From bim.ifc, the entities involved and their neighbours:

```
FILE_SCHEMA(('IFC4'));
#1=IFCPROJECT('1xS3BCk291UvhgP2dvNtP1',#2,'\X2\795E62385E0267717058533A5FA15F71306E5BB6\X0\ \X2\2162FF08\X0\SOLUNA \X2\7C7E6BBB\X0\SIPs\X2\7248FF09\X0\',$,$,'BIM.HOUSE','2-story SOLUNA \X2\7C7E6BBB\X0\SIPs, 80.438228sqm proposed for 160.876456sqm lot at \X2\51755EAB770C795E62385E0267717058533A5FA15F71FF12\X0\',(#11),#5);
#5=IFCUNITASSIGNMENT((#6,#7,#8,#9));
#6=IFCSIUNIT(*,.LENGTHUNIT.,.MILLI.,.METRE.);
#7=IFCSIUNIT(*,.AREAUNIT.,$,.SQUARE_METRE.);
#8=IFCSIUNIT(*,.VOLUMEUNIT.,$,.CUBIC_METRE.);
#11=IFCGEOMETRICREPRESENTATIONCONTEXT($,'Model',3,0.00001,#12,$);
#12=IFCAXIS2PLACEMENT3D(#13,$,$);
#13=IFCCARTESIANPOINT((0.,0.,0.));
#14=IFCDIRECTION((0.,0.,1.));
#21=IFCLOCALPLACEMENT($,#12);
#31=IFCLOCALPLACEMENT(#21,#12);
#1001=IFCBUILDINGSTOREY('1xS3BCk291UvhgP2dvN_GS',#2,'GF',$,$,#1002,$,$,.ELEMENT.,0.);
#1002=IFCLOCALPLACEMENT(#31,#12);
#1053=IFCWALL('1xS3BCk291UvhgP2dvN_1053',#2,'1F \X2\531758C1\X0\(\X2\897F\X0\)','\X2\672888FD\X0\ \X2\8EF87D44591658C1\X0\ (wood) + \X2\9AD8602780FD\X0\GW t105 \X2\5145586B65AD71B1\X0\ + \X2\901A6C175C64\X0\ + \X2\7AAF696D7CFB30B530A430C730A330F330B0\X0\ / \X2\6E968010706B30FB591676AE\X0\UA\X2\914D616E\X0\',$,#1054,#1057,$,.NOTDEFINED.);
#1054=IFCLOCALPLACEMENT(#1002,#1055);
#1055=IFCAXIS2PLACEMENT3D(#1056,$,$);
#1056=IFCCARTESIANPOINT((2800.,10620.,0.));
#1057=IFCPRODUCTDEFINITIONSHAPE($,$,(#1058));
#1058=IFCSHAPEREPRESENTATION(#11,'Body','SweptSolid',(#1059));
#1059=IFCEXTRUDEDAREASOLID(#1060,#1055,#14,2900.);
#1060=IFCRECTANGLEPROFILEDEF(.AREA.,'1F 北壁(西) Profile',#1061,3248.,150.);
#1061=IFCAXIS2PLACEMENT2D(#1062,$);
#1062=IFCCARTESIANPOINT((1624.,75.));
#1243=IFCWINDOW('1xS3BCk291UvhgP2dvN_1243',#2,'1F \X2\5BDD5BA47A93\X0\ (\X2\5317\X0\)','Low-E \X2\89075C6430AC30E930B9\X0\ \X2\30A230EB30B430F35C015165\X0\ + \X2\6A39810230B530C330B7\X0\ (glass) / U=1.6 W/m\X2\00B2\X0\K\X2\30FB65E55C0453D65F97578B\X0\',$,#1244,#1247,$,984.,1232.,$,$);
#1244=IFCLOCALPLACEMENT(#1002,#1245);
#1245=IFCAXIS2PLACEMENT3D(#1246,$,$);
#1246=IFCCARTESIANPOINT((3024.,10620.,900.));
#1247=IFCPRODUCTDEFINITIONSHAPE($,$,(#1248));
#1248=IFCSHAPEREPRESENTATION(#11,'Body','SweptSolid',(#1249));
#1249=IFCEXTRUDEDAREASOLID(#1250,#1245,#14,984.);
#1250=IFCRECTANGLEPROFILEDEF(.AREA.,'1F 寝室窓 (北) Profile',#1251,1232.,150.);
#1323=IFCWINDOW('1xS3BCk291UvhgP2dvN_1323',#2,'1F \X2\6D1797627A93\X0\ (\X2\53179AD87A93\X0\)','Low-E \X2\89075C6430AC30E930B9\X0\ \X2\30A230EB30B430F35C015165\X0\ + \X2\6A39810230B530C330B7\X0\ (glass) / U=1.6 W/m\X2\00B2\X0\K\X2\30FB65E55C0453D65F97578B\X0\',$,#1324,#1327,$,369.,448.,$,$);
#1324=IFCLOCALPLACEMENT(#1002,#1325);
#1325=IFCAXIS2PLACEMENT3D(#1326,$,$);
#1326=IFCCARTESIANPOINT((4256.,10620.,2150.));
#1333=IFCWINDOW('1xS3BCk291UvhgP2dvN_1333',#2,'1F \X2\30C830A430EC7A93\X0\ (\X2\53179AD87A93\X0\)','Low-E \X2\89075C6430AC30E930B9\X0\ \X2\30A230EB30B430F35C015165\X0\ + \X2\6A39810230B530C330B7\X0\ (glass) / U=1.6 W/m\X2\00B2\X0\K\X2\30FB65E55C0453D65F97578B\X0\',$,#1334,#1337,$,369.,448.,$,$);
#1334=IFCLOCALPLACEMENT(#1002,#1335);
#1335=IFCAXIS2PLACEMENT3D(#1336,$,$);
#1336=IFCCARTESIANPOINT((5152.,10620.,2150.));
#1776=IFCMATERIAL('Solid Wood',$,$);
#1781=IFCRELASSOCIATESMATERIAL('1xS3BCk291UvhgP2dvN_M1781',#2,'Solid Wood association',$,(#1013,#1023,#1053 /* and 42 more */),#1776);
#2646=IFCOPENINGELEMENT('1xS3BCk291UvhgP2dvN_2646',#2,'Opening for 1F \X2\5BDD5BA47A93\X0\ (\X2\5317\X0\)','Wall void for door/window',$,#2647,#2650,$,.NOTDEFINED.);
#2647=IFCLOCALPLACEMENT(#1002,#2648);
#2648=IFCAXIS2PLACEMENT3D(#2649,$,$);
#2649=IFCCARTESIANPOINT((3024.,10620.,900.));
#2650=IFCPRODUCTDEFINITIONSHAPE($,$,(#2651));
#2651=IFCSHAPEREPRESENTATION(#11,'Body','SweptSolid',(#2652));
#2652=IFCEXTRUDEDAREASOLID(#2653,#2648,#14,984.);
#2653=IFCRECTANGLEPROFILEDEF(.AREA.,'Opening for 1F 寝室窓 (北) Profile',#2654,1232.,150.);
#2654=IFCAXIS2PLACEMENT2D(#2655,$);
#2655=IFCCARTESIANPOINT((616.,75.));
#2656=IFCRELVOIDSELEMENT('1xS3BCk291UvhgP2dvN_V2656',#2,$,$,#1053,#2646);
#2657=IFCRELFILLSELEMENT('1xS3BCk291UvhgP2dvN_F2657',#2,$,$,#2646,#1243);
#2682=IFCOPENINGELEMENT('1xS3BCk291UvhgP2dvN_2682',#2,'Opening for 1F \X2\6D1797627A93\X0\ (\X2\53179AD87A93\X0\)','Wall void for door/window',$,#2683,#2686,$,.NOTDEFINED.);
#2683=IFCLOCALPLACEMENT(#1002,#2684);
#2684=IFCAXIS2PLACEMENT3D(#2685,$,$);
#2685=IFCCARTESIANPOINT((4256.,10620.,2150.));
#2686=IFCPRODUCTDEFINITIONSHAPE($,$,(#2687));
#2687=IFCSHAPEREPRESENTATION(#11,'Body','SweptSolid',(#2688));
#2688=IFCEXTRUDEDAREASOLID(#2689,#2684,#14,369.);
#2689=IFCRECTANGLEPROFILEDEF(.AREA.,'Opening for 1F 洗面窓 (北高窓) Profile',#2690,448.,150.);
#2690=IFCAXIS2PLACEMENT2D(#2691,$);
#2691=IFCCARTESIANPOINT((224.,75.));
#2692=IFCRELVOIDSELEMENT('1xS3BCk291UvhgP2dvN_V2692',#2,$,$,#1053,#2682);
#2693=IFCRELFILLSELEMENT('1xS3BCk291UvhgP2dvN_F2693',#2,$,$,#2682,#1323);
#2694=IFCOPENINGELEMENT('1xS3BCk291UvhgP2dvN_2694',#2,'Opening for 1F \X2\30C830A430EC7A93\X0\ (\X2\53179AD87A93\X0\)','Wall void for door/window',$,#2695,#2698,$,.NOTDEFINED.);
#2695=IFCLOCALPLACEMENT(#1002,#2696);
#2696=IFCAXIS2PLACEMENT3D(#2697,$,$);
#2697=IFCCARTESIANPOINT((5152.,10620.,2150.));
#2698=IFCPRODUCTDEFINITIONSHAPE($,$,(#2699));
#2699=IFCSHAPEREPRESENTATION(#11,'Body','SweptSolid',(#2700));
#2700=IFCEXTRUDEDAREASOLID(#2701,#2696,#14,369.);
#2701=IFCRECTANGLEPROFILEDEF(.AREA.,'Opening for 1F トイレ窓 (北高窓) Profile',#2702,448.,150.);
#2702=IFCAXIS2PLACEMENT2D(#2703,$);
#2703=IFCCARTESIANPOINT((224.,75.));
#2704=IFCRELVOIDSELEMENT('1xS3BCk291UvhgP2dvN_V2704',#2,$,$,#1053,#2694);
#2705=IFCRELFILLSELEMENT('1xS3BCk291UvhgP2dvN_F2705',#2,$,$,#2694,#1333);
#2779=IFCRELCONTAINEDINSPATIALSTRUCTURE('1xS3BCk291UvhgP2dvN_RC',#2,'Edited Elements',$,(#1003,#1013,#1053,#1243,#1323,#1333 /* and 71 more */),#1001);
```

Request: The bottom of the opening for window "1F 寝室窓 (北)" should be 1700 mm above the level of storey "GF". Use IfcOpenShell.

```python
import numpy as np
import ifcopenshell
import ifcopenshell.api.geometry
import ifcopenshell.geom
import ifcopenshell.util.element
import ifcopenshell.util.placement
import ifcopenshell.util.shape
import ifcopenshell.util.unit

model = ifcopenshell.open("bim.ifc")
unit_scale = ifcopenshell.util.unit.calculate_unit_scale(model)

window = model.by_guid("1xS3BCk291UvhgP2dvN_1243")
opening = window.FillsVoids[0].RelatingOpeningElement
storey = ifcopenshell.util.element.get_container(window, ifc_class="IfcBuildingStorey")
level = ifcopenshell.util.placement.get_local_placement(storey.ObjectPlacement)[2, 3]

# The opening's origin need not be at the sill, so measure its lowest point.
shape = ifcopenshell.geom.create_shape(ifcopenshell.geom.settings(), opening)
bottom = ifcopenshell.util.shape.get_shape_bottom_elevation(shape, shape.geometry) / unit_scale
dz = level + 1.7 / unit_scale - bottom

shift = np.array([0.0, 0.0, dz])
# The window is not placed relative to its opening, so move both.
for product in (opening, window):
    matrix = ifcopenshell.util.placement.get_local_placement(product.ObjectPlacement)
    matrix[:3, 3] += shift
    ifcopenshell.api.geometry.edit_object_placement(model, product=product, matrix=matrix, is_si=False)

print(f"moved by {dz * unit_scale:+.3f} m")

model.write("bim_edited.ifc")
```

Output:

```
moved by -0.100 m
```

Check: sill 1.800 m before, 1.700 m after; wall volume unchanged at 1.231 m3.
